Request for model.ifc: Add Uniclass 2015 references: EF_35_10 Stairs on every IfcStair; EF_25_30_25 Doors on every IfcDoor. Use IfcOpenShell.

First a look at what the model holds.

```python
import ifcopenshell

model = ifcopenshell.open("model.ifc")
print(model.schema)
print("classifications:", [c.Name for c in model.by_type("IfcClassification")])
for ifc_class in ("IfcDoor", "IfcRoof", "IfcStair", "IfcWall", "IfcWindow"):
    print(ifc_class, len(model.by_type(ifc_class)))
```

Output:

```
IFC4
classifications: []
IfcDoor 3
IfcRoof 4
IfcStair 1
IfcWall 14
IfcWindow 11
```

```python
import ifcopenshell
import ifcopenshell.api.classification

model = ifcopenshell.open("model.ifc")

system = ifcopenshell.api.classification.add_classification(model, classification="Uniclass 2015")

codes = {
    "IfcStair": ("EF_35_10", "Stairs"),
    "IfcDoor": ("EF_25_30_25", "Doors"),
}
for ifc_class, (code, name) in codes.items():
    products = model.by_type(ifc_class)
    ifcopenshell.api.classification.add_reference(
        model, products=products, classification=system, identification=code, name=name
    )
    print(code, len(products))

model.write("model-out.ifc")
```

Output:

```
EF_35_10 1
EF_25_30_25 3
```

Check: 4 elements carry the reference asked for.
